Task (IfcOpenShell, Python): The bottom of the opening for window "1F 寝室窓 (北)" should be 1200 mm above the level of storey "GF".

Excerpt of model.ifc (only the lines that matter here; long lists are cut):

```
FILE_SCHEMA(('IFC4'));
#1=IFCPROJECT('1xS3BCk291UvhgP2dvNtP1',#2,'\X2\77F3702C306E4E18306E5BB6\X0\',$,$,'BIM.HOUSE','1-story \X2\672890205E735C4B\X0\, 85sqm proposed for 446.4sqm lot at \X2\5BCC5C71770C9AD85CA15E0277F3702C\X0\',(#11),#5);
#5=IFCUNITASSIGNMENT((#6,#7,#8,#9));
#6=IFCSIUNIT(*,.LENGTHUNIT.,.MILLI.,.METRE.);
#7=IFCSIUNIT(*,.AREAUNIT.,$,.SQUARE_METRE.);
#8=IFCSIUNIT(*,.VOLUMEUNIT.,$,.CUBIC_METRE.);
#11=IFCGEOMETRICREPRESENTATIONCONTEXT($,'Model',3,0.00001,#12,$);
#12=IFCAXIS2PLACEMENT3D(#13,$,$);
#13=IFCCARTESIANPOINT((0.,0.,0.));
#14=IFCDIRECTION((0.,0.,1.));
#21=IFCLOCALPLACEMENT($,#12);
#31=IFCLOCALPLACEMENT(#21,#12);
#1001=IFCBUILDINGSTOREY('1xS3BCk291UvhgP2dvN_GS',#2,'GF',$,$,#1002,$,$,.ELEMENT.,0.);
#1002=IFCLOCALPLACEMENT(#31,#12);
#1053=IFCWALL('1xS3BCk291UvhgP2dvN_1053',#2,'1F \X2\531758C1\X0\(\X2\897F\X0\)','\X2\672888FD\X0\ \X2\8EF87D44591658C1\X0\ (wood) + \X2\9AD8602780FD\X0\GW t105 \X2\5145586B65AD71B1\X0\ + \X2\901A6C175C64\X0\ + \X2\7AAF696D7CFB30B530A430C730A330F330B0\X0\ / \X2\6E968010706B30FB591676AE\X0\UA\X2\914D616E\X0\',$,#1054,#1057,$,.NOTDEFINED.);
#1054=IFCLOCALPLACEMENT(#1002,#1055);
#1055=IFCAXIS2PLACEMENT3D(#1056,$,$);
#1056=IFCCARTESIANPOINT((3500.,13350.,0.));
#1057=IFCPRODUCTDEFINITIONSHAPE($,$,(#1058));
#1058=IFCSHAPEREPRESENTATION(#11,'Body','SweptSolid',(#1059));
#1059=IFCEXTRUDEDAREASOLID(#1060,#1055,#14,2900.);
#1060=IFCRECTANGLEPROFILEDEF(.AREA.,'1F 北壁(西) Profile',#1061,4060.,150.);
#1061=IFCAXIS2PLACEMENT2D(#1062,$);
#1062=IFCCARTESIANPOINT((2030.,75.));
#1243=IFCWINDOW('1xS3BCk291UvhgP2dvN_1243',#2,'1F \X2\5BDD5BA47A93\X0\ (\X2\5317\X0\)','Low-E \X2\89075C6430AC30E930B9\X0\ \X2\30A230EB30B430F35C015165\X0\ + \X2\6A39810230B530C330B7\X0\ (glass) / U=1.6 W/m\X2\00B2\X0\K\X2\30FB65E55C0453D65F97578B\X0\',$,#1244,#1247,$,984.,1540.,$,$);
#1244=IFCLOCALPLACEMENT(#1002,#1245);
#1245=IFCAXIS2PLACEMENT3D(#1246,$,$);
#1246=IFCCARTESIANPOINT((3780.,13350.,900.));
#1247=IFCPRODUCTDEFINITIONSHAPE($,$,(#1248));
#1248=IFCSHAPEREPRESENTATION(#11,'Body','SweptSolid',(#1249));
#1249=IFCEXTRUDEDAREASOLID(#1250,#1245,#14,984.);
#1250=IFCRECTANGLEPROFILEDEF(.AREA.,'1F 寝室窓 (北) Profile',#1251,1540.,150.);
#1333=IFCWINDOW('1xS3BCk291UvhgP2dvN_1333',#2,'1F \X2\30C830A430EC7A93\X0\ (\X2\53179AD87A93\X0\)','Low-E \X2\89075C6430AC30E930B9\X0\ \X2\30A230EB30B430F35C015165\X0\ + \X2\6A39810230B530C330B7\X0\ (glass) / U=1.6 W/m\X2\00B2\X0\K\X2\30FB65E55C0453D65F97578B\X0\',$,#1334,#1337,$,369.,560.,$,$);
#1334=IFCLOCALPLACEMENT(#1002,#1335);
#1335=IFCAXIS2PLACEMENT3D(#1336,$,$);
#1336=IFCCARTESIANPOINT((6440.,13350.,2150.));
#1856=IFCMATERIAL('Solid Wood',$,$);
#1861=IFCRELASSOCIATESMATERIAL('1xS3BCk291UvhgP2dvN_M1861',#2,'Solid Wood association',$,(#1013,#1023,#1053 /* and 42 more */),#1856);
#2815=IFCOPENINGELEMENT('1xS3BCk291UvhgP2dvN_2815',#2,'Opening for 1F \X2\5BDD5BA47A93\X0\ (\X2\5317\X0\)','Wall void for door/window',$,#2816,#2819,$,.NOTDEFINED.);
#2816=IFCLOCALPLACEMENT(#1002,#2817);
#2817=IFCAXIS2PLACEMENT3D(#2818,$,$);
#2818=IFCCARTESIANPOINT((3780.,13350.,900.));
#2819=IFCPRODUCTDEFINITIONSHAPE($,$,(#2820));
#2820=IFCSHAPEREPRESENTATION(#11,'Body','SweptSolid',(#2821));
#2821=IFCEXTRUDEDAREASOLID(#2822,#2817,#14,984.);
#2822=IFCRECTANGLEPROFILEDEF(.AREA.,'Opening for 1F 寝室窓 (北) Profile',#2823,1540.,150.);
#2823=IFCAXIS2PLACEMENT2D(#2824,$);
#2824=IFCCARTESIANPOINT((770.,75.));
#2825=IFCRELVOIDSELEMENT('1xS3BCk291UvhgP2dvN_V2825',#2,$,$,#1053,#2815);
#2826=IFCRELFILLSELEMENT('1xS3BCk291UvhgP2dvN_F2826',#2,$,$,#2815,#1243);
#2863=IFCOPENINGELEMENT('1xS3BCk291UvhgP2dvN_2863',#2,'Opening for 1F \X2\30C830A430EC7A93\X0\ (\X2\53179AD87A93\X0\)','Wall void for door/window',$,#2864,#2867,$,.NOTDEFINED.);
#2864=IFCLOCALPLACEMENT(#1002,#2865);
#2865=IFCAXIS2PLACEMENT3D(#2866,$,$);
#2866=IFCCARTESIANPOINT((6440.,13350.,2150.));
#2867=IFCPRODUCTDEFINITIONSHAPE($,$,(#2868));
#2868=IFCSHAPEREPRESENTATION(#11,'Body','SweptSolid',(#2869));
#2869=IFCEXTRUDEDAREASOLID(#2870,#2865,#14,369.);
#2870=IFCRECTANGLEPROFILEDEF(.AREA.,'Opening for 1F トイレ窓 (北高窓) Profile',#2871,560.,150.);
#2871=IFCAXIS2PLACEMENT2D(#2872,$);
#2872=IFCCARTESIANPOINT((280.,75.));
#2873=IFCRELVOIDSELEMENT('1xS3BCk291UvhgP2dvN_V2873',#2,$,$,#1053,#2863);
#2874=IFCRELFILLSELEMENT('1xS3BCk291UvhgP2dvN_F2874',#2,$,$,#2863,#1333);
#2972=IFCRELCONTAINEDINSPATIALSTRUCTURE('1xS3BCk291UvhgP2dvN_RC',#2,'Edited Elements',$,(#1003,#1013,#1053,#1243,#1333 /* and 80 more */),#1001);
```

```python
import numpy as np
import ifcopenshell
import ifcopenshell.api.geometry
import ifcopenshell.geom
import ifcopenshell.util.element
import ifcopenshell.util.placement
import ifcopenshell.util.shape
import ifcopenshell.util.unit

model = ifcopenshell.open("model.ifc")
unit_scale = ifcopenshell.util.unit.calculate_unit_scale(model)

window = model.by_guid("1xS3BCk291UvhgP2dvN_1243")
opening = window.FillsVoids[0].RelatingOpeningElement
storey = ifcopenshell.util.element.get_container(window, ifc_class="IfcBuildingStorey")
level = ifcopenshell.util.placement.get_local_placement(storey.ObjectPlacement)[2, 3]

# The opening's origin need not be at the sill, so measure its lowest point.
shape = ifcopenshell.geom.create_shape(ifcopenshell.geom.settings(), opening)
bottom = ifcopenshell.util.shape.get_shape_bottom_elevation(shape, shape.geometry) / unit_scale
dz = level + 1.2 / unit_scale - bottom

shift = np.array([0.0, 0.0, dz])
# The window is not placed relative to its opening, so move both.
for product in (opening, window):
    matrix = ifcopenshell.util.placement.get_local_placement(product.ObjectPlacement)
    matrix[:3, 3] += shift
    ifcopenshell.api.geometry.edit_object_placement(model, product=product, matrix=matrix, is_si=False)

print(f"moved by {dz * unit_scale:+.3f} m")

model.write("model_edited.ifc")
```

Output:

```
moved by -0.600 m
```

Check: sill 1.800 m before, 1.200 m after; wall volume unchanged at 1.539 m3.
